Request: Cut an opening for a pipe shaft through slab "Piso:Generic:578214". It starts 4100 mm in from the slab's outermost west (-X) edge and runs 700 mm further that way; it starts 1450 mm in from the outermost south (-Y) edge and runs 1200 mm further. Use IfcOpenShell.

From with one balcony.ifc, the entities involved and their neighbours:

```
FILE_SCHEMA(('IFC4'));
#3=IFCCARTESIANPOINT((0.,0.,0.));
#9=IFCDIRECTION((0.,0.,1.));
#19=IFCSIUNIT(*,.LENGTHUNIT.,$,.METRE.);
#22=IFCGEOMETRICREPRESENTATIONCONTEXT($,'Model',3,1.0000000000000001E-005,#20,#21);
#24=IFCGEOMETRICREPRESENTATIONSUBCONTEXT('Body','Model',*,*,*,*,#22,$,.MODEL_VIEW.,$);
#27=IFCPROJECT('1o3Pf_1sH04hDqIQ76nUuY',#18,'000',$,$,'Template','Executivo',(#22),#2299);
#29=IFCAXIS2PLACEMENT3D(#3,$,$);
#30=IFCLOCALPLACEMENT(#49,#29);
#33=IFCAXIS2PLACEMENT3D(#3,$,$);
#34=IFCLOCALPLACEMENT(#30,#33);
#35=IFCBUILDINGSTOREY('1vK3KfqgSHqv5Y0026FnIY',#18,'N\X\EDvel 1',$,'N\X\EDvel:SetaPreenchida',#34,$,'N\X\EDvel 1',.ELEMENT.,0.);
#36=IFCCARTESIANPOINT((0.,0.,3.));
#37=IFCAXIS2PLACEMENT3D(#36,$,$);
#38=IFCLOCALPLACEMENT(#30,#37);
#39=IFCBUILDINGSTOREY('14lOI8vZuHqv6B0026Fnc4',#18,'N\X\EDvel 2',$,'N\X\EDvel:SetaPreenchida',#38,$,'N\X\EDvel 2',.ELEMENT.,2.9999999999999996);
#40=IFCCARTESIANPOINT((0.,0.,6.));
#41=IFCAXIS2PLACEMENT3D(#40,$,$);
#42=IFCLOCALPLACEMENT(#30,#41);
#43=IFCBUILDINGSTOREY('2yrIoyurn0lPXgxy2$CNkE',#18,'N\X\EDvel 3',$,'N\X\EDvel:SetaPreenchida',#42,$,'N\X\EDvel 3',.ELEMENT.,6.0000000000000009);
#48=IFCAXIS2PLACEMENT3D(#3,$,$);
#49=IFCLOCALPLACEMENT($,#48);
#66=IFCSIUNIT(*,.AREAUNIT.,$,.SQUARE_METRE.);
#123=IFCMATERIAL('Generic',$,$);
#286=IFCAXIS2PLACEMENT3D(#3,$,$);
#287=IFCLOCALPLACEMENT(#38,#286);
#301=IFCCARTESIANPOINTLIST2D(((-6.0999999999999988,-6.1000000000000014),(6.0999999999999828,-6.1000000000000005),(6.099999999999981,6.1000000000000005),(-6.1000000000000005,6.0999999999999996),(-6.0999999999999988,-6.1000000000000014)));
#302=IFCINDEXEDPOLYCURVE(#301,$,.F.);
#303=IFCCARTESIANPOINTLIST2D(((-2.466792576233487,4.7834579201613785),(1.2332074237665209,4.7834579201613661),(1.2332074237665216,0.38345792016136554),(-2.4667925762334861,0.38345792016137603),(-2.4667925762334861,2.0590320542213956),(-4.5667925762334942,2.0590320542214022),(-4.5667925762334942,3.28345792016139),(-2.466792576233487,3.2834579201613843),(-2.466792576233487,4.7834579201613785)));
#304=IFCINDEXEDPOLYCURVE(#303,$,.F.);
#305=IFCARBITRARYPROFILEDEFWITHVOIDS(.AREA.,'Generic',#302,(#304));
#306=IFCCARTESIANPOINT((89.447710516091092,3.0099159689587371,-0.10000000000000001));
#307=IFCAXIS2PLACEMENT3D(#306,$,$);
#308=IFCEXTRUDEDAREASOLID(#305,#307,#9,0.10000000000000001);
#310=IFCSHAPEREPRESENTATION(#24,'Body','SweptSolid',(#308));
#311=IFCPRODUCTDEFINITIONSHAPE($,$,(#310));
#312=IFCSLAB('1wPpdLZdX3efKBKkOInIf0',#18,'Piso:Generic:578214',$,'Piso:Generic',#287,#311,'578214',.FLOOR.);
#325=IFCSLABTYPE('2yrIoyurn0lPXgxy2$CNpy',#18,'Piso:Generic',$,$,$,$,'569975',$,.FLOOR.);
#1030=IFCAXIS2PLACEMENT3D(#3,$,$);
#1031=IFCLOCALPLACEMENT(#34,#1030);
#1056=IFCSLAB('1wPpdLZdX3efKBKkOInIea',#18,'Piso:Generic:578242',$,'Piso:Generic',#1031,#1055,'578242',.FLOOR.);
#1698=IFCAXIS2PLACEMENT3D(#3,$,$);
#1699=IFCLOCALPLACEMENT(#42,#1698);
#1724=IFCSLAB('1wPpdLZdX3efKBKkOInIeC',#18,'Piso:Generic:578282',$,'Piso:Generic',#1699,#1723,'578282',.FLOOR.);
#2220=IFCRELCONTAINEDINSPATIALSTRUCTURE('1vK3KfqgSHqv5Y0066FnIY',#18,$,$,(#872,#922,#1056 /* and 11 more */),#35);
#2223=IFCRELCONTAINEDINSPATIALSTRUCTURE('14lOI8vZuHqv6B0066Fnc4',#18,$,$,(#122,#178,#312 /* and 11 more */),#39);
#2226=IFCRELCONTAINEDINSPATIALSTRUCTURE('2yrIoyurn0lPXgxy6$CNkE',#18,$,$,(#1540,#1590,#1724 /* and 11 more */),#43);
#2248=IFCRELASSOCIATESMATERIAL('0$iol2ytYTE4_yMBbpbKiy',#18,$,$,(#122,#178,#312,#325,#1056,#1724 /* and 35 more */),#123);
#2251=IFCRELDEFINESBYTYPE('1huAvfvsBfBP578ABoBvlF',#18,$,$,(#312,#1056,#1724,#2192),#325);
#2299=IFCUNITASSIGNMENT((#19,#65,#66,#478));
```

```python
import numpy as np
import ifcopenshell
import ifcopenshell.api.feature
import ifcopenshell.api.geometry
import ifcopenshell.api.root
import ifcopenshell.geom
import ifcopenshell.util.placement
import ifcopenshell.util.representation
import ifcopenshell.util.shape
import ifcopenshell.util.unit

model = ifcopenshell.open("with one balcony.ifc")
unit_scale = ifcopenshell.util.unit.calculate_unit_scale(model)
settings = ifcopenshell.geom.settings()


def volume(element):
    """Net volume in cubic metres, openings subtracted."""
    shape = ifcopenshell.geom.create_shape(settings, element)
    return ifcopenshell.util.shape.get_volume(shape.geometry)


slab = model.by_guid("1wPpdLZdX3efKBKkOInIf0")
before = volume(slab)

# Extent in the slab's own axes, in metres. The edges named are its -X and -Y sides.
slab_shape = ifcopenshell.geom.create_shape(settings, slab)
vertices = ifcopenshell.util.shape.get_vertices(slab_shape.geometry)
x_min, y_min, bottom = vertices.min(axis=0)
top = vertices[:, 2].max()

opening = ifcopenshell.api.root.create_entity(model, ifc_class="IfcOpeningElement", name="Pipe shaft opening", predefined_type="OPENING")
context = ifcopenshell.util.representation.get_context(model, "Model", "Body", "MODEL_VIEW")
width, depth = 0.7, 1.2
outline = [(0.0, 0.0), (width, 0.0), (width, depth), (0.0, depth), (0.0, 0.0)]
# Overshoot both faces by 50 mm so the cut is clean.
shape = ifcopenshell.api.geometry.add_slab_representation(
    model, context=context, depth=top - bottom + 0.1, polyline=outline
)
ifcopenshell.api.geometry.assign_representation(model, product=opening, representation=shape)

matrix = ifcopenshell.util.placement.get_local_placement(slab.ObjectPlacement)
matrix[:, 3] = matrix @ np.append(np.array([x_min + 4.1, y_min + 1.45, bottom - 0.05]) / unit_scale, 1.0)
ifcopenshell.api.geometry.edit_object_placement(model, product=opening, matrix=matrix, is_si=False)
ifcopenshell.api.feature.add_feature(model, feature=opening, element=slab)

after = volume(slab)

print(f"slab volume {before:.3f} -> {after:.3f} m3")

model.write("with one balcony-out.ifc")
```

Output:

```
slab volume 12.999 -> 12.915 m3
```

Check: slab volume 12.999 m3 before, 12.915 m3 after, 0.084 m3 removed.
